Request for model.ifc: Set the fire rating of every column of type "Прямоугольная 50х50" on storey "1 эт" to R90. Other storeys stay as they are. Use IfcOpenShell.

First a look at what the model holds.

```python
import ifcopenshell
import ifcopenshell.util.element

model = ifcopenshell.open("model.ifc")
print(model.schema)
storey = next(s for s in model.by_type("IfcBuildingStorey") if s.Name == "1 эт")
columns = [e for e in ifcopenshell.util.element.get_decomposition(storey) if e.is_a("IfcColumn")]
seen = {}
for e in columns:
    element_type = ifcopenshell.util.element.get_type(e)
    key = (element_type.Name if element_type != e and element_type else None, ifcopenshell.util.element.get_pset(e, "Pset_ColumnCommon", "FireRating"))
    seen[key] = seen.get(key, 0) + 1
for (name, value), count in sorted(seen.items(), key=str):
    print(count, "x", name, "|", value)
```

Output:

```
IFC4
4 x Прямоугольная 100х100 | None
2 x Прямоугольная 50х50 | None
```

```python
import ifcopenshell
import ifcopenshell.api.pset
import ifcopenshell.util.element

model = ifcopenshell.open("model.ifc")

storey = next(s for s in model.by_type("IfcBuildingStorey") if s.Name == "1 эт")
columns = [e for e in ifcopenshell.util.element.get_decomposition(storey) if e.is_a("IfcColumn")]

count = 0
for e in columns:
    element_type = ifcopenshell.util.element.get_type(e)
    if element_type in (None, e) or element_type.Name != "Прямоугольная 50х50":
        continue
    # add_pset returns the element's existing set when there is one.
    pset = ifcopenshell.api.pset.add_pset(model, product=e, name="Pset_ColumnCommon")
    ifcopenshell.api.pset.edit_pset(model, pset=pset, properties={"FireRating": "R90"})
    count += 1

print(count, "columns updated")

model.write("model_edited.ifc")
```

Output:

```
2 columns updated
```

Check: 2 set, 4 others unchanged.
